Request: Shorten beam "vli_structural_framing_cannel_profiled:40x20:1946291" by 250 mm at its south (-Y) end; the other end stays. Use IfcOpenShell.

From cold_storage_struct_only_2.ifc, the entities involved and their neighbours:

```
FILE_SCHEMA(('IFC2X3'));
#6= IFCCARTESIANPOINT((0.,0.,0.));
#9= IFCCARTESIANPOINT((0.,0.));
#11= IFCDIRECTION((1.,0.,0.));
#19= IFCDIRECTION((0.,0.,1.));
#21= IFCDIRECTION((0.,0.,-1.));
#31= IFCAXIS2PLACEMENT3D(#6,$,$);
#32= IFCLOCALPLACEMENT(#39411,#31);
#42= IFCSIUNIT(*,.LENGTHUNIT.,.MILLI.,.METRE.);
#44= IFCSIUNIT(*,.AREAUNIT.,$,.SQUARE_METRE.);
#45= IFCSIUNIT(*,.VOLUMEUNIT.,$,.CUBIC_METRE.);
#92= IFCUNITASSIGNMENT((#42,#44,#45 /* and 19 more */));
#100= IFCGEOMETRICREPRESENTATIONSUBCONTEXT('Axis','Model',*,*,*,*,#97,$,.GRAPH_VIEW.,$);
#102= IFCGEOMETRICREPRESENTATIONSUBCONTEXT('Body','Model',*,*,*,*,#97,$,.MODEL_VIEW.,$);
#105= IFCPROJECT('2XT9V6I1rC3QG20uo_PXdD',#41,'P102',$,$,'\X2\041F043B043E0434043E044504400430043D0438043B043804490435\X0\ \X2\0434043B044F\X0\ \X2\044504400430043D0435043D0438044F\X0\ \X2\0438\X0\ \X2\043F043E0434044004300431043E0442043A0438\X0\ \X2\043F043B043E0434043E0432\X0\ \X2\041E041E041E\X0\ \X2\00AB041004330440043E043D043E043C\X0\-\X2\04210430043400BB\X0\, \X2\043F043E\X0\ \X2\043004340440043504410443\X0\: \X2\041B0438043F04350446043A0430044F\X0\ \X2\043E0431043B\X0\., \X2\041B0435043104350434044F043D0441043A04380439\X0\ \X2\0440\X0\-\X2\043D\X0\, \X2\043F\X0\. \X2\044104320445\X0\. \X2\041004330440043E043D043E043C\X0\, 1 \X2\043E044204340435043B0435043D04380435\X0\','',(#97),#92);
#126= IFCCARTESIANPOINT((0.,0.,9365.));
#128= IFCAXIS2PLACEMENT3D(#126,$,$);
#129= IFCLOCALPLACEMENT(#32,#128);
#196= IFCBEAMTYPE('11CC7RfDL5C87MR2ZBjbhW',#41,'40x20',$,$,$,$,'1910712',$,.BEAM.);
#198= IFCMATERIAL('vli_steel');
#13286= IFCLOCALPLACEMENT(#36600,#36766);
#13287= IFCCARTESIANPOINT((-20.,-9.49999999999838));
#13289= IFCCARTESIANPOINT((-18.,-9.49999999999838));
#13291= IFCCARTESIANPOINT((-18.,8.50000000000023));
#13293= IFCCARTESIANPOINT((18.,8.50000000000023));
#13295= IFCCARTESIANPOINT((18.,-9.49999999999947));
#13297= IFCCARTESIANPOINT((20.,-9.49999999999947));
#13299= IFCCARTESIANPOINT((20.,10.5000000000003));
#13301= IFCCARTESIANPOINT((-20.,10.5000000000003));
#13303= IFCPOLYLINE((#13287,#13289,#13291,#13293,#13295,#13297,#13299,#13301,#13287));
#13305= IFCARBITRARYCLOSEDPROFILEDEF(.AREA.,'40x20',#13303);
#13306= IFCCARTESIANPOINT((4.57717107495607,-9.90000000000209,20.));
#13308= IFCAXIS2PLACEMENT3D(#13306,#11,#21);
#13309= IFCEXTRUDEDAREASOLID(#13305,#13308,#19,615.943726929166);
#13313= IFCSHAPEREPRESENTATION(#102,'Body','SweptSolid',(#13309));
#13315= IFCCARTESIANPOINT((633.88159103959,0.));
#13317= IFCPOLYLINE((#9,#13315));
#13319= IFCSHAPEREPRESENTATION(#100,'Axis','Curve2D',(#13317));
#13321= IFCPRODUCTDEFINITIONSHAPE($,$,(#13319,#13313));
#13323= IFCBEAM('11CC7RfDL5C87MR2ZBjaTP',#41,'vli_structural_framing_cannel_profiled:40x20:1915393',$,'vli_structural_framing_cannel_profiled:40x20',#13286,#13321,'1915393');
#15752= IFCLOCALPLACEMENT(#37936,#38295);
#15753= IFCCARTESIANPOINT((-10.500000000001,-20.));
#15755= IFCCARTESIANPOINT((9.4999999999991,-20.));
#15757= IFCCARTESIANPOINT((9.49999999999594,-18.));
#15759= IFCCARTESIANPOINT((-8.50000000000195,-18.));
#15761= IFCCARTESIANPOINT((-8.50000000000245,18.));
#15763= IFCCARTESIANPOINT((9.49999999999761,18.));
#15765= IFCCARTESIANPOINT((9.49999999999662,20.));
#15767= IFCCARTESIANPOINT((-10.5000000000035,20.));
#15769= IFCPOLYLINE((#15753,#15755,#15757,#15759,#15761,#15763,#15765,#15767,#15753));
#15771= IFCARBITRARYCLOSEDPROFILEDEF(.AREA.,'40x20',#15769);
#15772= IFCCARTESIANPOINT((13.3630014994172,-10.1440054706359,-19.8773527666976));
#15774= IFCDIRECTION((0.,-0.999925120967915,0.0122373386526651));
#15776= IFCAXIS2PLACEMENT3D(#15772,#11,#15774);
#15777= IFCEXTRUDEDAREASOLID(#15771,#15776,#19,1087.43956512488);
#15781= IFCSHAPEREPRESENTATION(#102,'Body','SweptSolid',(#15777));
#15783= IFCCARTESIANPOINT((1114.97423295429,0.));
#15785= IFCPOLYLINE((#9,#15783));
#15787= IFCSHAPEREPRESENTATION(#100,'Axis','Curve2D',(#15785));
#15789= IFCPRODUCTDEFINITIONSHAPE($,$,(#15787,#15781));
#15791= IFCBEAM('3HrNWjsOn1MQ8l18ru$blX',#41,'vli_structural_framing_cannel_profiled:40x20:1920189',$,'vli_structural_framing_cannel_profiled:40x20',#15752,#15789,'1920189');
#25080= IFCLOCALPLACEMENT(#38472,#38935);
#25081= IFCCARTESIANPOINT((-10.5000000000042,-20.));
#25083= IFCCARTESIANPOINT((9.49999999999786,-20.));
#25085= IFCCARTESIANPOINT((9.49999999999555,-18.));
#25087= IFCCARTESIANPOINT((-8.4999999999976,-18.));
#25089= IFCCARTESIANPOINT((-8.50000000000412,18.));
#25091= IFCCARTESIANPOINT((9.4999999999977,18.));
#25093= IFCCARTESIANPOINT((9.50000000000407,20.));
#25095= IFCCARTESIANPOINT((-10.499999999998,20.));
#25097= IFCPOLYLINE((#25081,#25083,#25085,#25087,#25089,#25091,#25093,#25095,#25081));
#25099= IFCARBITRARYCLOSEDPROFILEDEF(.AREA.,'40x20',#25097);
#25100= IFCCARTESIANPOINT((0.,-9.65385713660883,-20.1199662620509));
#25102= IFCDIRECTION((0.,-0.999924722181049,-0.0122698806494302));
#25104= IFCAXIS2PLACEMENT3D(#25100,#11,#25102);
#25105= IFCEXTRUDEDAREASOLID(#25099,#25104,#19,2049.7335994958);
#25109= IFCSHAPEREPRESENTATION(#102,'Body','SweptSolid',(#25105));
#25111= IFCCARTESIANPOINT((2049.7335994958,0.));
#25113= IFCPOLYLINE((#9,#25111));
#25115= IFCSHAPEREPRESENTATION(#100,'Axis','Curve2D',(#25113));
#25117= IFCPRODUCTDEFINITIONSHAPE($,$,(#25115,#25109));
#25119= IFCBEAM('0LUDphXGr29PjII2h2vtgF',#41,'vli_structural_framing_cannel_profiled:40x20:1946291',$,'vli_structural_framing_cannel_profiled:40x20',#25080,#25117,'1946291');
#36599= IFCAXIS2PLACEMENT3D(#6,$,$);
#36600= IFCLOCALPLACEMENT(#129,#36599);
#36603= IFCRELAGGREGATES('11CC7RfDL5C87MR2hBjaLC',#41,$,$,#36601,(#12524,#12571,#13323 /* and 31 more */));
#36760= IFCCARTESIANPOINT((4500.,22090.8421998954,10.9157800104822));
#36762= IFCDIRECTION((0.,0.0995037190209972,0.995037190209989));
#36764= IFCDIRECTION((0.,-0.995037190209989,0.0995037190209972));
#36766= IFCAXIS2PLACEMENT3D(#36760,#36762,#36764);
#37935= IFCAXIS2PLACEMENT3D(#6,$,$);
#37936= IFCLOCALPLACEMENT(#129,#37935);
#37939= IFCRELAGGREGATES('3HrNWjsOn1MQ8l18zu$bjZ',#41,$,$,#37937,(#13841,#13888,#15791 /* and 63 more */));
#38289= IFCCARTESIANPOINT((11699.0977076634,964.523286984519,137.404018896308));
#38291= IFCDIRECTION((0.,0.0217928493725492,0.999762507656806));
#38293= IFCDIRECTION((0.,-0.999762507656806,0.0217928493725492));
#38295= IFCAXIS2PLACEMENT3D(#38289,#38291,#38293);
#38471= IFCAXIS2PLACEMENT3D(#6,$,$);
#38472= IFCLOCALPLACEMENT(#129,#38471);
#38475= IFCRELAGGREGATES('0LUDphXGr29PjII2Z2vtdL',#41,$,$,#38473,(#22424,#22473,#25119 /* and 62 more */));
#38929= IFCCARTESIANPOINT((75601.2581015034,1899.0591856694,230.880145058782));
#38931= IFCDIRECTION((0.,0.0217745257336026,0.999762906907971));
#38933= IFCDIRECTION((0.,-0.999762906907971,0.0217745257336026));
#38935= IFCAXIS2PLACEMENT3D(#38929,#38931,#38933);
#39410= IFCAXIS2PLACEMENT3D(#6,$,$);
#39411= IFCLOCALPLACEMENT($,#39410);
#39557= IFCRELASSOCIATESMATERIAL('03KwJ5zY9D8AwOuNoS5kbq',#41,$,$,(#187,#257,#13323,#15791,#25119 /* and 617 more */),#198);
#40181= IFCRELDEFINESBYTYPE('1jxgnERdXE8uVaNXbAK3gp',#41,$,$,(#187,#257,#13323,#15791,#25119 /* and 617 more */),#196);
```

```python
import numpy as np
import ifcopenshell
import ifcopenshell.util.representation

model = ifcopenshell.open("cold_storage_struct_only_2.ifc")

member = model.by_guid("0LUDphXGr29PjII2h2vtgF")
change = -250.0

# The extrusion runs towards the end named, so only its depth changes.
body = ifcopenshell.util.representation.get_representation(member, "Model", "Body")
solid = body.Items[0]
old_length = solid.Depth
solid.Depth += change

# Move the axis end point with it.
axis = next(r for r in member.Representation.Representations if r.RepresentationIdentifier == "Axis").Items[0]
start, end = (np.array(p.Coordinates) for p in axis.Points)
end = end + (end - start) / np.linalg.norm(end - start) * change
point = model.createIfcCartesianPoint(end.tolist())
axis.Points = [axis.Points[0], point]

print(f"length {old_length:g} -> {solid.Depth:g}")

model.write("cold_storage_struct_only_2_edited.ifc")
```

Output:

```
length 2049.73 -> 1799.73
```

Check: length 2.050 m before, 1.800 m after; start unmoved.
